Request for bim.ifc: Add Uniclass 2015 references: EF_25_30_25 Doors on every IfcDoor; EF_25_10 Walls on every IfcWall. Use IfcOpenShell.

First a look at what the model holds.

```python
import ifcopenshell

model = ifcopenshell.open("bim.ifc")
print(model.schema)
print("classifications:", [c.Name for c in model.by_type("IfcClassification")])
for ifc_class in ("IfcDoor", "IfcRoof", "IfcStair", "IfcWall", "IfcWindow"):
    print(ifc_class, len(model.by_type(ifc_class)))
```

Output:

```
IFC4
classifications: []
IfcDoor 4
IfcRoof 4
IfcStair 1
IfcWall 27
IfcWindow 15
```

```python
import ifcopenshell
import ifcopenshell.api.classification

model = ifcopenshell.open("bim.ifc")

system = ifcopenshell.api.classification.add_classification(model, classification="Uniclass 2015")

codes = {
    "IfcDoor": ("EF_25_30_25", "Doors"),
    "IfcWall": ("EF_25_10", "Walls"),
}
for ifc_class, (code, name) in codes.items():
    products = model.by_type(ifc_class)
    ifcopenshell.api.classification.add_reference(
        model, products=products, classification=system, identification=code, name=name
    )
    print(code, len(products))

model.write("bim_updated.ifc")
```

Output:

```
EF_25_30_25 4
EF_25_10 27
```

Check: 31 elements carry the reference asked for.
